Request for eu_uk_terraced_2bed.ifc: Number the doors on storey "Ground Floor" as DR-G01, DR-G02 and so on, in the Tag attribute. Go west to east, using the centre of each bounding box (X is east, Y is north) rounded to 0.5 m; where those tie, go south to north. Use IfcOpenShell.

First a look at what the model holds.

```python
import ifcopenshell
import ifcopenshell.util.element
import ifcopenshell.util.placement

model = ifcopenshell.open("eu_uk_terraced_2bed.ifc")
print(model.schema)
storey = next(s for s in model.by_type("IfcBuildingStorey") if s.Name == "Ground Floor")
doors = [e for e in ifcopenshell.util.element.get_decomposition(storey) if e.is_a("IfcDoor")]
for e in sorted(doors, key=lambda e: e.id()):
    origin = ifcopenshell.util.placement.get_local_placement(e.ObjectPlacement)[:3, 3]
    print(e.id(), e.Tag, e.Name, origin.round(2) + 0.0, sep=" | ")
```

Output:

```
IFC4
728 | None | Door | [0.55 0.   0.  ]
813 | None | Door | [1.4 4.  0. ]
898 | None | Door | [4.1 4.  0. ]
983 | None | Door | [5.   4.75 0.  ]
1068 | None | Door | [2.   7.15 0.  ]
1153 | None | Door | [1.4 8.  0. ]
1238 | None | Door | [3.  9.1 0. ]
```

```python
import ifcopenshell
import ifcopenshell.geom
import ifcopenshell.util.element
import ifcopenshell.util.shape

model = ifcopenshell.open("eu_uk_terraced_2bed.ifc")
settings = ifcopenshell.geom.settings()
settings.set("use-world-coords", True)


def centre(element):
    shape = ifcopenshell.geom.create_shape(settings, element)
    return ifcopenshell.util.shape.get_bbox_centroid(shape.geometry)


storey = next(s for s in model.by_type("IfcBuildingStorey") if s.Name == "Ground Floor")
doors = [e for e in ifcopenshell.util.element.get_decomposition(storey) if e.is_a("IfcDoor")]

# Insertion points can sit at a corner or the storey origin, so sort by the geometry (in metres).
centres = {e: centre(e) for e in doors}
doors.sort(key=lambda e: (round(centres[e][0] / 0.5), centres[e][1]))

for i, e in enumerate(doors, start=1):
    number = f"DR-G{i:02d}"
    e.Tag = number
    print(e.id(), number)

model.write("eu_uk_terraced_2bed_rev.ifc")
```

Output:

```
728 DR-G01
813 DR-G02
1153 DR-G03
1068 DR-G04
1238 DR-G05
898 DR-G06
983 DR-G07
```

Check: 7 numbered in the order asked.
